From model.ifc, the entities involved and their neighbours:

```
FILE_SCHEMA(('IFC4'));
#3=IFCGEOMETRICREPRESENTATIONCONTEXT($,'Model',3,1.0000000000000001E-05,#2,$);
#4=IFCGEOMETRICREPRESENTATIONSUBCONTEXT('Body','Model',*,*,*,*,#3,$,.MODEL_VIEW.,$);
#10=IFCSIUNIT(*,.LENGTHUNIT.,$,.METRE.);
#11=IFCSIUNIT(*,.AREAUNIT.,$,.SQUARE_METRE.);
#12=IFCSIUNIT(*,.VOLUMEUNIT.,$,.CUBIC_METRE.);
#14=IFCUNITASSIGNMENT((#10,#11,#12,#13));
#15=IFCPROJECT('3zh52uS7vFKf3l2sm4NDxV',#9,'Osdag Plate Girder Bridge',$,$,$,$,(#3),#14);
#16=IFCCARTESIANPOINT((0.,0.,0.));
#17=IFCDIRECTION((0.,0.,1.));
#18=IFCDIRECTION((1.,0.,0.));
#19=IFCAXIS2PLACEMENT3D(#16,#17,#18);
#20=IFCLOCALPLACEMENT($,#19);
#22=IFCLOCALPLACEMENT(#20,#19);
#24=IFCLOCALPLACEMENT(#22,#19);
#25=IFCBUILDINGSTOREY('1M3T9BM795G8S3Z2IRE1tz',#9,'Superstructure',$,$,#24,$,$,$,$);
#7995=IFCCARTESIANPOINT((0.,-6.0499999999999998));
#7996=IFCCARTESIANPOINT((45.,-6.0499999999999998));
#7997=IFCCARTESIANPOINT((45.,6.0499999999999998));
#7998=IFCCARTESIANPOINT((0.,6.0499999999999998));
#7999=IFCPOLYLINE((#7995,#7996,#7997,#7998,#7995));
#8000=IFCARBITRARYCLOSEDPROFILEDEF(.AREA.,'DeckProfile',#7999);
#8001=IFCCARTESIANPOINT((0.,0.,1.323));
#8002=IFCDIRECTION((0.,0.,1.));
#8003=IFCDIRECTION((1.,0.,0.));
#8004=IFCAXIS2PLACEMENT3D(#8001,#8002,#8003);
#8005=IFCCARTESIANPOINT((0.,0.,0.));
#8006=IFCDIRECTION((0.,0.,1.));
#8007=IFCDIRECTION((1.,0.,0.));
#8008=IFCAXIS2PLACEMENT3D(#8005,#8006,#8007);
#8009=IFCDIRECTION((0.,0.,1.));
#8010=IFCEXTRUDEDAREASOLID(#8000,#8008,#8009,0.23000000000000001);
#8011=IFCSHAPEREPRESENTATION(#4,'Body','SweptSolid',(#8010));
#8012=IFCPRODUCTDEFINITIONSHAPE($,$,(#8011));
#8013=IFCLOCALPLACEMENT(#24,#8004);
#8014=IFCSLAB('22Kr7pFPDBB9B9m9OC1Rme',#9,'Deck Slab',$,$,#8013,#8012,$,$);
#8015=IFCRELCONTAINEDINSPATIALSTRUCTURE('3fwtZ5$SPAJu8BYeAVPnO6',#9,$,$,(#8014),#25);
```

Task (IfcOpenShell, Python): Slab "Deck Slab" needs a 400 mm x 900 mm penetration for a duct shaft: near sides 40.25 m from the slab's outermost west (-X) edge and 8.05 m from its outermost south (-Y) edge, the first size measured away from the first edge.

```python
import numpy as np
import ifcopenshell
import ifcopenshell.api.feature
import ifcopenshell.api.geometry
import ifcopenshell.api.root
import ifcopenshell.geom
import ifcopenshell.util.placement
import ifcopenshell.util.representation
import ifcopenshell.util.shape
import ifcopenshell.util.unit

model = ifcopenshell.open("model.ifc")
unit_scale = ifcopenshell.util.unit.calculate_unit_scale(model)
settings = ifcopenshell.geom.settings()


def volume(element):
    """Net volume in cubic metres, openings subtracted."""
    shape = ifcopenshell.geom.create_shape(settings, element)
    return ifcopenshell.util.shape.get_volume(shape.geometry)


slab = model.by_guid("22Kr7pFPDBB9B9m9OC1Rme")
before = volume(slab)

# Extent in the slab's own axes, in metres. The edges named are its -X and -Y sides.
slab_shape = ifcopenshell.geom.create_shape(settings, slab)
vertices = ifcopenshell.util.shape.get_vertices(slab_shape.geometry)
x_min, y_min, bottom = vertices.min(axis=0)
top = vertices[:, 2].max()

opening = ifcopenshell.api.root.create_entity(model, ifc_class="IfcOpeningElement", name="Duct shaft opening", predefined_type="OPENING")
context = ifcopenshell.util.representation.get_context(model, "Model", "Body", "MODEL_VIEW")
width, depth = 0.4, 0.9
outline = [(0.0, 0.0), (width, 0.0), (width, depth), (0.0, depth), (0.0, 0.0)]
# Overshoot both faces by 50 mm so the cut is clean.
shape = ifcopenshell.api.geometry.add_slab_representation(
    model, context=context, depth=top - bottom + 0.1, polyline=outline
)
ifcopenshell.api.geometry.assign_representation(model, product=opening, representation=shape)

matrix = ifcopenshell.util.placement.get_local_placement(slab.ObjectPlacement)
matrix[:, 3] = matrix @ np.append(np.array([x_min + 40.25, y_min + 8.05, bottom - 0.05]) / unit_scale, 1.0)
ifcopenshell.api.geometry.edit_object_placement(model, product=opening, matrix=matrix, is_si=False)
ifcopenshell.api.feature.add_feature(model, feature=opening, element=slab)

after = volume(slab)

print(f"slab volume {before:.3f} -> {after:.3f} m3")

model.write("model_edited.ifc")
```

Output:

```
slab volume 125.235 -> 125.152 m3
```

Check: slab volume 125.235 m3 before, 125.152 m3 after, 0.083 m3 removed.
